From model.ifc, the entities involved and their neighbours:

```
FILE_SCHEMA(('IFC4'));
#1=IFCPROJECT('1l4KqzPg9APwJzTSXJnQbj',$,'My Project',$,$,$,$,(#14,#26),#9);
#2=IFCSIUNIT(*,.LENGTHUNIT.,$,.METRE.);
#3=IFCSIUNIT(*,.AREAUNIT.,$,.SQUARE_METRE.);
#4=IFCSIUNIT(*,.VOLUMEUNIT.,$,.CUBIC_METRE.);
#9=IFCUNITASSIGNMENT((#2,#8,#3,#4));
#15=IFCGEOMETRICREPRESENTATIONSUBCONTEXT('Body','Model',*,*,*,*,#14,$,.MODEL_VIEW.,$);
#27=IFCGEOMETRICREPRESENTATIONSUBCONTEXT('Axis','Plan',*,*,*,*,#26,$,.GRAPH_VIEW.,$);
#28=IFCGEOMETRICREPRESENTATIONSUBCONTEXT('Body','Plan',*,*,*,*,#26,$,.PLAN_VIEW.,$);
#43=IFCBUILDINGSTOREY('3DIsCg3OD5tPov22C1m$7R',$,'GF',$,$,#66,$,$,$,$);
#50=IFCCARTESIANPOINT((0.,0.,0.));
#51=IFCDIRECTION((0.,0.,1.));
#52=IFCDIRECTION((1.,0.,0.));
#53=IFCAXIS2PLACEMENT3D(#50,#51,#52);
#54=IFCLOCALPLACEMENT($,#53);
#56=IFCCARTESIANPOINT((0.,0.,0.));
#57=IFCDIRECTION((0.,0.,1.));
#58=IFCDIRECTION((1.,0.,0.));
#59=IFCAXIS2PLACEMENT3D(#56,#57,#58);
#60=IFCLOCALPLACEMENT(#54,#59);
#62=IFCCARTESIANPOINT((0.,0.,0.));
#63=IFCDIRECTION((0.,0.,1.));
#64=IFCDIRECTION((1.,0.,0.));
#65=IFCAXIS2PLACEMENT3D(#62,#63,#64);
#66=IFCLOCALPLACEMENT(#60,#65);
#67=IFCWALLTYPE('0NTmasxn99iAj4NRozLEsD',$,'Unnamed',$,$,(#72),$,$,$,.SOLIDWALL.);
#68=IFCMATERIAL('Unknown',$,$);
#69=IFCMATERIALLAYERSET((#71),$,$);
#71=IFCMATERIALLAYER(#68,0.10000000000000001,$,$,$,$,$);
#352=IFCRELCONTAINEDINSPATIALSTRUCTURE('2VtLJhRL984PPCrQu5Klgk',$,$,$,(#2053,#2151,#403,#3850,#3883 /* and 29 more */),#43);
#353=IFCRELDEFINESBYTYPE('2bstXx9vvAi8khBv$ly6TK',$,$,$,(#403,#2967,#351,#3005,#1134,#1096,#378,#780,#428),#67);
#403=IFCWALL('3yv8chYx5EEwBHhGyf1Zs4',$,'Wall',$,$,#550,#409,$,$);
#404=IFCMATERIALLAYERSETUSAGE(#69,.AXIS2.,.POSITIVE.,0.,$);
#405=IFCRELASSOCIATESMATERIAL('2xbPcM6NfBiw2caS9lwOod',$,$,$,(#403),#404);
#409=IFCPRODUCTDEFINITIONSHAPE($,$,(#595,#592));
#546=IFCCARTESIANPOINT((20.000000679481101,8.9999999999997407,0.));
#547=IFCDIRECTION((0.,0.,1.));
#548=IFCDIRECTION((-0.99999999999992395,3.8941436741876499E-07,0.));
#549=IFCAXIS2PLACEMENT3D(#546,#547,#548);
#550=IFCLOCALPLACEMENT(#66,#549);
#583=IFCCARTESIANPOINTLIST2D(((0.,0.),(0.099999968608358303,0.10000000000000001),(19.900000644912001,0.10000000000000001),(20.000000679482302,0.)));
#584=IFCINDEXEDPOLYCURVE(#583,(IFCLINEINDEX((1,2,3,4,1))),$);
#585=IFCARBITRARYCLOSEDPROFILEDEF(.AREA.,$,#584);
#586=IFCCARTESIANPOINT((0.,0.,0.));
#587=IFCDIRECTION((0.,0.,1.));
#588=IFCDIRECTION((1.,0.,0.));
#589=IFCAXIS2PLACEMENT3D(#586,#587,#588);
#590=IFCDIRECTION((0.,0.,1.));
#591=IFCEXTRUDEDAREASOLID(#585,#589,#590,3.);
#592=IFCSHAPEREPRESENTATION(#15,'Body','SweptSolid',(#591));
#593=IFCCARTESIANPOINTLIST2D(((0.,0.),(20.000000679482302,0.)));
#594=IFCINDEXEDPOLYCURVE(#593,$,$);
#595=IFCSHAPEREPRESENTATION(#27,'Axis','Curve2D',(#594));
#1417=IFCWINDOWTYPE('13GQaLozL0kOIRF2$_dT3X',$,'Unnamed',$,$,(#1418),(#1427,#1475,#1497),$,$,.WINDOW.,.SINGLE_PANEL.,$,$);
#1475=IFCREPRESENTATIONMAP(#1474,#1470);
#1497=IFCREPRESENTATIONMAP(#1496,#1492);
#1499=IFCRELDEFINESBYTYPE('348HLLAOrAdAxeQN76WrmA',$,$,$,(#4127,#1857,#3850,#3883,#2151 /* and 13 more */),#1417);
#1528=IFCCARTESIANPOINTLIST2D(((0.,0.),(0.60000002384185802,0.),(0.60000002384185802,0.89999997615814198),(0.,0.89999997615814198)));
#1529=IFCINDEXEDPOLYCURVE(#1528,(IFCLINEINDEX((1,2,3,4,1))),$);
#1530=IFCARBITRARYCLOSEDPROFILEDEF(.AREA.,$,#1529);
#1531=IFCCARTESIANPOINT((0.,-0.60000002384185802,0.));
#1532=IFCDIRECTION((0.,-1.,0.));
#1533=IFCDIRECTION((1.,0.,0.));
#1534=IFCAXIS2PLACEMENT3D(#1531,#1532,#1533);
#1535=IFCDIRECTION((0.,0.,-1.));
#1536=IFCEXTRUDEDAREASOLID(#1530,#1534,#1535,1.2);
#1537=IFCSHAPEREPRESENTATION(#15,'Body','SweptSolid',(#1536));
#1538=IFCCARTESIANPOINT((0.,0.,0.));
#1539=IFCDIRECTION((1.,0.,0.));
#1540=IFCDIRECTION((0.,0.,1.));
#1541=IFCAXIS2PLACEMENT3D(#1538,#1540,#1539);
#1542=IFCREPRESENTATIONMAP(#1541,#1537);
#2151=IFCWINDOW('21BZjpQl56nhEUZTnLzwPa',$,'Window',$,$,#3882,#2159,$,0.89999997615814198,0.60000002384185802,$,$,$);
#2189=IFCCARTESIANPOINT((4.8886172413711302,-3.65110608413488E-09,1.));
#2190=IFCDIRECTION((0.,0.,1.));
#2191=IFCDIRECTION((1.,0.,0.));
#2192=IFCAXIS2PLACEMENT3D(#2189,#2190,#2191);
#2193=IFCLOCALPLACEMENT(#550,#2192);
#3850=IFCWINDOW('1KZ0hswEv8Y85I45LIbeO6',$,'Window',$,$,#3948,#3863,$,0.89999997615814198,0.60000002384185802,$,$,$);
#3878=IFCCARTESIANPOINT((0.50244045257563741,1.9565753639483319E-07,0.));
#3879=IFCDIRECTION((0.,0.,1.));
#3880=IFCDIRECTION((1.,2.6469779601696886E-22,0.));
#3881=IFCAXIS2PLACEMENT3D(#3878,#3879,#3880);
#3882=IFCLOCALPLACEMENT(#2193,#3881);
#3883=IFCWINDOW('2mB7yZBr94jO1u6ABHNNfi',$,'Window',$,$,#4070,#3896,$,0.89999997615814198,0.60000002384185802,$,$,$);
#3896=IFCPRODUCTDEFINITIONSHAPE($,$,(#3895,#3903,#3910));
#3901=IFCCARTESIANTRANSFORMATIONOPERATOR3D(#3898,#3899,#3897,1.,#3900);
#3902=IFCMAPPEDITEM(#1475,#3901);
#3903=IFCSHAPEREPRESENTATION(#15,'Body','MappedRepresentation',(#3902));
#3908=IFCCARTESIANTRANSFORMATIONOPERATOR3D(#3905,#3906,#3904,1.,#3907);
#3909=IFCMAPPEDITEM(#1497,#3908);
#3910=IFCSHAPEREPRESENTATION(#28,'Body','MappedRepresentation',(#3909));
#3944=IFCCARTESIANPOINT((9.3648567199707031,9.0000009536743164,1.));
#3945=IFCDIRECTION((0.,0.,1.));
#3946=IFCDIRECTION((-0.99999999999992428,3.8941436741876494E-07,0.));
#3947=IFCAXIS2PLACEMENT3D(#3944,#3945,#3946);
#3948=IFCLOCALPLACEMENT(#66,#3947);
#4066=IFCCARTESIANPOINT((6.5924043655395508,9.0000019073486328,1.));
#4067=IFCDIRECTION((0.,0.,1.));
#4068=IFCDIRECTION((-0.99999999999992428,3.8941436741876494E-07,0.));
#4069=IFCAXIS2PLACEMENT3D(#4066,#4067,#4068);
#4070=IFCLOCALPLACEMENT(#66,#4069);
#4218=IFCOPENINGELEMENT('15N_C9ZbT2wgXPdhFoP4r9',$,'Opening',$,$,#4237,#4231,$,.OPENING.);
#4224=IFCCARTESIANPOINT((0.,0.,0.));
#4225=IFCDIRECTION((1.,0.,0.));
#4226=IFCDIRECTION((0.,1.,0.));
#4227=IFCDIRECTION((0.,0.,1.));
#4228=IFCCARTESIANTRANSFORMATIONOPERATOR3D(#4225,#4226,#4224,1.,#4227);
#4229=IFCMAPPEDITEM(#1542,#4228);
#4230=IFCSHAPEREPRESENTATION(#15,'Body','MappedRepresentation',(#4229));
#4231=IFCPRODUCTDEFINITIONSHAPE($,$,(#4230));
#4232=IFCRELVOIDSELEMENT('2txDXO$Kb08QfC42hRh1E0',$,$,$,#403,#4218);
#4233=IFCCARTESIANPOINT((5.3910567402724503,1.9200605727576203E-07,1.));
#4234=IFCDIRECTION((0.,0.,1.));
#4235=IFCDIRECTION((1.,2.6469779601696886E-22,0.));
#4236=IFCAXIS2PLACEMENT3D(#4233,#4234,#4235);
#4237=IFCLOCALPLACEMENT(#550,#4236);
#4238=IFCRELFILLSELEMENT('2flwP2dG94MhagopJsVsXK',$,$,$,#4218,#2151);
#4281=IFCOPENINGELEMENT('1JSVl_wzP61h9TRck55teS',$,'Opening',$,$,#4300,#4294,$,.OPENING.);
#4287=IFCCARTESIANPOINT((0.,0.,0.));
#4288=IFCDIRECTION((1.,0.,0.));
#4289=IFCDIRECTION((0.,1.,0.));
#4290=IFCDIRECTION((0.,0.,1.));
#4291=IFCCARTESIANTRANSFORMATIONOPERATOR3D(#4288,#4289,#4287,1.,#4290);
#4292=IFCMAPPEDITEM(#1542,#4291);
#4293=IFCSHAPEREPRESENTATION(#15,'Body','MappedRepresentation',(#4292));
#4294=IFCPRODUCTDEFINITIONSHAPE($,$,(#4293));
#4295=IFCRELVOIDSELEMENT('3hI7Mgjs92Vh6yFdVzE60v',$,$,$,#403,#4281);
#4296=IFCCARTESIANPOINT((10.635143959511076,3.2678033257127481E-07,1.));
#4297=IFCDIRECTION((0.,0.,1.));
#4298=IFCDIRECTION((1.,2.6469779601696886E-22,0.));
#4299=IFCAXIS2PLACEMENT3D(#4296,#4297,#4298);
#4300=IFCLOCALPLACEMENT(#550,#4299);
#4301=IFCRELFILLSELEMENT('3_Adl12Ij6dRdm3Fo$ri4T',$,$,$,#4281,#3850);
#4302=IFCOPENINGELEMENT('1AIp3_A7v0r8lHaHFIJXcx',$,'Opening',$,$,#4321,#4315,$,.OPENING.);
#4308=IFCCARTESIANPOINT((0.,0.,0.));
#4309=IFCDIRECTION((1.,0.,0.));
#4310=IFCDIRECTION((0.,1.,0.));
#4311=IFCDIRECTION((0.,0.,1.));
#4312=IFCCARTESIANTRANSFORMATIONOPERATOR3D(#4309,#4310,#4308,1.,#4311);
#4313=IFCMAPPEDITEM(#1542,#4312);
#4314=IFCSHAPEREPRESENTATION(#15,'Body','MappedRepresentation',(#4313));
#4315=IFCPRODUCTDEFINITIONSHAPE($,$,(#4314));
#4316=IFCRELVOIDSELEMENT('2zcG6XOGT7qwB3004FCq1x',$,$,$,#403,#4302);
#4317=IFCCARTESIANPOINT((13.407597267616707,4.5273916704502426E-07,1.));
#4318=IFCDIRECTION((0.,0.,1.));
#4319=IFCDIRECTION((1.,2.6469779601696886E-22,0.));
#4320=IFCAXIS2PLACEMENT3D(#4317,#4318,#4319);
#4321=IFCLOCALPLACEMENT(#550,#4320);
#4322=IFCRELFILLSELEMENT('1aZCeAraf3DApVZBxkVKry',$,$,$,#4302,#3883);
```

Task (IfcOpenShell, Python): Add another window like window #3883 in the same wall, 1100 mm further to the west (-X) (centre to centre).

```python
import ifcopenshell
import ifcopenshell.api.feature
import ifcopenshell.api.geometry
import ifcopenshell.api.root
import ifcopenshell.geom
import ifcopenshell.util.element
import ifcopenshell.util.placement
import ifcopenshell.util.shape
import ifcopenshell.util.unit

model = ifcopenshell.open("model.ifc")
unit_scale = ifcopenshell.util.unit.calculate_unit_scale(model)
settings = ifcopenshell.geom.settings()


def volume(element):
    """Net volume in cubic metres, openings subtracted."""
    shape = ifcopenshell.geom.create_shape(settings, element)
    return ifcopenshell.util.shape.get_volume(shape.geometry)


window = model.by_id(3883)
opening = window.FillsVoids[0].RelatingOpeningElement
wall = opening.VoidsElements[0].RelatingBuildingElement
before = volume(wall)
shift = ifcopenshell.util.placement.get_local_placement(wall.ObjectPlacement)[:3, 0] * 1.1 / unit_scale

# copy_class copies the void relationship, type, container and properties, but no geometry.
new_opening = ifcopenshell.api.root.copy_class(model, product=opening)
new_opening.Representation = ifcopenshell.util.element.copy_deep(
    model, opening.Representation, exclude=["IfcGeometricRepresentationContext", "IfcRepresentationMap"]
)
new_window = ifcopenshell.api.root.copy_class(model, product=window)
new_window.Representation = ifcopenshell.util.element.copy_deep(
    model, window.Representation, exclude=["IfcGeometricRepresentationContext", "IfcRepresentationMap"]
)
ifcopenshell.api.feature.add_filling(model, opening=new_opening, element=new_window)

for old, new in ((opening, new_opening), (window, new_window)):
    matrix = ifcopenshell.util.placement.get_local_placement(old.ObjectPlacement)
    matrix[:3, 3] += shift
    ifcopenshell.api.geometry.edit_object_placement(model, product=new, matrix=matrix, is_si=False)

after = volume(wall)

print(f"wall volume {before:.3f} -> {after:.3f} m3")

model.write("model-out.ifc")
```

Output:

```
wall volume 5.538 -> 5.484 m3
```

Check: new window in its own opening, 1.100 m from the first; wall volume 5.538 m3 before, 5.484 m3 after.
